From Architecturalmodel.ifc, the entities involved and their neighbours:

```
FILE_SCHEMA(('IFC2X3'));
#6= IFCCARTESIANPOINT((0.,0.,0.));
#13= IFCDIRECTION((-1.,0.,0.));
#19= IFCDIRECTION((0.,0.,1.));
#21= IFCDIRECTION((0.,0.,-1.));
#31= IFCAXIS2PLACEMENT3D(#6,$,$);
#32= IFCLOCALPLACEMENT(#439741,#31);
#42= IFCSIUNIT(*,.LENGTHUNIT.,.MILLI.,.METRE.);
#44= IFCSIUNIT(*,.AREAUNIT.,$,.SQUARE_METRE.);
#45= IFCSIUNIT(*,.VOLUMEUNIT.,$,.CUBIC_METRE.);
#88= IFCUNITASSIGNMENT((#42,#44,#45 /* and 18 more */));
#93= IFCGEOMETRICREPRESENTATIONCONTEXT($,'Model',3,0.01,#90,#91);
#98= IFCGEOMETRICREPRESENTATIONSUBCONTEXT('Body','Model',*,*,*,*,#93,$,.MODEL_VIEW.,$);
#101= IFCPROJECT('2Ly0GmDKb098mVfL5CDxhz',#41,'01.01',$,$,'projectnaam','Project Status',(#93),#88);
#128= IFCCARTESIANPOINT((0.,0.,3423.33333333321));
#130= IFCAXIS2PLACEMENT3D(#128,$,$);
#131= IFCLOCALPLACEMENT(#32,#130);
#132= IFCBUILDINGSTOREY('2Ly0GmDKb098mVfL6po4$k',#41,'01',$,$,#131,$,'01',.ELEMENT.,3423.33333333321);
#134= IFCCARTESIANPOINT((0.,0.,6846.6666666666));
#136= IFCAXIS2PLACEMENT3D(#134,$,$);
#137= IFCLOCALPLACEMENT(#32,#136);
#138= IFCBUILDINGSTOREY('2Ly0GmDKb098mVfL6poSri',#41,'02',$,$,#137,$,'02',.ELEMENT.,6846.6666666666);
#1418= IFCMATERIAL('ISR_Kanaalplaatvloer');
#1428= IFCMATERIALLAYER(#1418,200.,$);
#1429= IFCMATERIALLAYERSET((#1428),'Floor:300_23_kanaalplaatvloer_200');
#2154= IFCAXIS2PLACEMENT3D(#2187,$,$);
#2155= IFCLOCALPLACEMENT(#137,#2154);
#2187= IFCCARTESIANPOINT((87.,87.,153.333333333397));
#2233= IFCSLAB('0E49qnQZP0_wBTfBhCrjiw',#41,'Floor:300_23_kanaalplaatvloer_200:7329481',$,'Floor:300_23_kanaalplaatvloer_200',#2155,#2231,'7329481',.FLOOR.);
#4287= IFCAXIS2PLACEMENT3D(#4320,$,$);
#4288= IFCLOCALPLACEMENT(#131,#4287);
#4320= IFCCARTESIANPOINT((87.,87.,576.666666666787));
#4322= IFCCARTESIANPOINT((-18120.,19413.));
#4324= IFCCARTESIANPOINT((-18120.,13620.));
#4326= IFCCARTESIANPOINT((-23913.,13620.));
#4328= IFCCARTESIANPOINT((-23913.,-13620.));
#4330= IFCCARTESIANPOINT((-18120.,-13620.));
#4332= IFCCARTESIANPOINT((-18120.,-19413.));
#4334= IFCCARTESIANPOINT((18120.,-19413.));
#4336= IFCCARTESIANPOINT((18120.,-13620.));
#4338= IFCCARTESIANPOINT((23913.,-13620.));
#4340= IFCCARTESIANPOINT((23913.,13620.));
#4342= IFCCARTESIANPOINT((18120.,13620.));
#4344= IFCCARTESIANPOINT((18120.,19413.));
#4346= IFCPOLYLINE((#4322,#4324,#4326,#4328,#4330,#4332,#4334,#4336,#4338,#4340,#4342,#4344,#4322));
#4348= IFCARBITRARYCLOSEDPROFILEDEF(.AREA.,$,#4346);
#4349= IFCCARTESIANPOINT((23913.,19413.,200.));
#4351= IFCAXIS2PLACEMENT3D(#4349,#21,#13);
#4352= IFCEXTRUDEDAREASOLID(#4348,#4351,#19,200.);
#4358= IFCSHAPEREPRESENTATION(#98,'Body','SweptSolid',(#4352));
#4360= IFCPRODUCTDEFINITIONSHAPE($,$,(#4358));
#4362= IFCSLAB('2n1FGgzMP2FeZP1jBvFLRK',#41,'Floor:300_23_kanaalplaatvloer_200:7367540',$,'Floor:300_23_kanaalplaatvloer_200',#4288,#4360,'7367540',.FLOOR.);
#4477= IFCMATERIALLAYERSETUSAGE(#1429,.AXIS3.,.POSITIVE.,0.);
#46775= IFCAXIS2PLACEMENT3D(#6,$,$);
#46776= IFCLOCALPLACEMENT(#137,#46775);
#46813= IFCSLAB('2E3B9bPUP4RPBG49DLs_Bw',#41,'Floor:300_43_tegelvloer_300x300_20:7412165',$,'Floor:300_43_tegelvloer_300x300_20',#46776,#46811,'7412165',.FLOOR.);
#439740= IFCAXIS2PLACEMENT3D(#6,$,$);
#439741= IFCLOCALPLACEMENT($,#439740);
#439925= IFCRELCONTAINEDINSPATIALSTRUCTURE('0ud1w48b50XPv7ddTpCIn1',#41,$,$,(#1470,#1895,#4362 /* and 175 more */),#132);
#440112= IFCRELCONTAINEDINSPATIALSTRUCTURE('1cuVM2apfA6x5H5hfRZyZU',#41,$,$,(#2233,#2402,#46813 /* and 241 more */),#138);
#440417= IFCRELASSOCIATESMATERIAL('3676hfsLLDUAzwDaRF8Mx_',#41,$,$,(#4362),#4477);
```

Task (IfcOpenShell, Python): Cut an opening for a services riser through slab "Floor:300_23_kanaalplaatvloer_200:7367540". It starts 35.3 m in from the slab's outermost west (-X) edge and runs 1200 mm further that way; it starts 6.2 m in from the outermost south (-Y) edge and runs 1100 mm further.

```python
import numpy as np
import ifcopenshell
import ifcopenshell.api.feature
import ifcopenshell.api.geometry
import ifcopenshell.api.root
import ifcopenshell.geom
import ifcopenshell.util.placement
import ifcopenshell.util.representation
import ifcopenshell.util.shape
import ifcopenshell.util.unit

model = ifcopenshell.open("Architecturalmodel.ifc")
unit_scale = ifcopenshell.util.unit.calculate_unit_scale(model)
settings = ifcopenshell.geom.settings()


def volume(element):
    """Net volume in cubic metres, openings subtracted."""
    shape = ifcopenshell.geom.create_shape(settings, element)
    return ifcopenshell.util.shape.get_volume(shape.geometry)


slab = model.by_guid("2n1FGgzMP2FeZP1jBvFLRK")
before = volume(slab)

# Extent in the slab's own axes, in metres. The edges named are its -X and -Y sides.
slab_shape = ifcopenshell.geom.create_shape(settings, slab)
vertices = ifcopenshell.util.shape.get_vertices(slab_shape.geometry)
x_min, y_min, bottom = vertices.min(axis=0)
top = vertices[:, 2].max()

opening = ifcopenshell.api.root.create_entity(model, ifc_class="IfcOpeningElement", name="Services riser opening")
context = ifcopenshell.util.representation.get_context(model, "Model", "Body", "MODEL_VIEW")
width, depth = 1.2, 1.1
outline = [(0.0, 0.0), (width, 0.0), (width, depth), (0.0, depth), (0.0, 0.0)]
# Overshoot both faces by 50 mm so the cut is clean.
shape = ifcopenshell.api.geometry.add_slab_representation(
    model, context=context, depth=top - bottom + 0.1, polyline=outline
)
ifcopenshell.api.geometry.assign_representation(model, product=opening, representation=shape)

matrix = ifcopenshell.util.placement.get_local_placement(slab.ObjectPlacement)
matrix[:, 3] = matrix @ np.append(np.array([x_min + 35.3, y_min + 6.2, bottom - 0.05]) / unit_scale, 1.0)
ifcopenshell.api.geometry.edit_object_placement(model, product=opening, matrix=matrix, is_si=False)
ifcopenshell.api.feature.add_feature(model, feature=opening, element=slab)

after = volume(slab)

print(f"slab volume {before:.3f} -> {after:.3f} m3")

model.write("Architecturalmodel_rev.ifc")
```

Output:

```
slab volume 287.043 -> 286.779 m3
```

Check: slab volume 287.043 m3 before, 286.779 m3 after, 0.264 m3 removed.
